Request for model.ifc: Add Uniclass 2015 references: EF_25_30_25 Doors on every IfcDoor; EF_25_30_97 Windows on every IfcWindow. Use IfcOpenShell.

First a look at what the model holds.

```python
import ifcopenshell

model = ifcopenshell.open("model.ifc")
print(model.schema)
print("classifications:", [c.Name for c in model.by_type("IfcClassification")])
for ifc_class in ("IfcDoor", "IfcRoof", "IfcStair", "IfcWall", "IfcWindow"):
    print(ifc_class, len(model.by_type(ifc_class)))
```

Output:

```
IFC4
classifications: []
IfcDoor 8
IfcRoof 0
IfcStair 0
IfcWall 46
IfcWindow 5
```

```python
import ifcopenshell
import ifcopenshell.api.classification

model = ifcopenshell.open("model.ifc")

system = ifcopenshell.api.classification.add_classification(model, classification="Uniclass 2015")

codes = {
    "IfcDoor": ("EF_25_30_25", "Doors"),
    "IfcWindow": ("EF_25_30_97", "Windows"),
}
for ifc_class, (code, name) in codes.items():
    products = model.by_type(ifc_class)
    ifcopenshell.api.classification.add_reference(
        model, products=products, classification=system, identification=code, name=name
    )
    print(code, len(products))

model.write("model_v2.ifc")
```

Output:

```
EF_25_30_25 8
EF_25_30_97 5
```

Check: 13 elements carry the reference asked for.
